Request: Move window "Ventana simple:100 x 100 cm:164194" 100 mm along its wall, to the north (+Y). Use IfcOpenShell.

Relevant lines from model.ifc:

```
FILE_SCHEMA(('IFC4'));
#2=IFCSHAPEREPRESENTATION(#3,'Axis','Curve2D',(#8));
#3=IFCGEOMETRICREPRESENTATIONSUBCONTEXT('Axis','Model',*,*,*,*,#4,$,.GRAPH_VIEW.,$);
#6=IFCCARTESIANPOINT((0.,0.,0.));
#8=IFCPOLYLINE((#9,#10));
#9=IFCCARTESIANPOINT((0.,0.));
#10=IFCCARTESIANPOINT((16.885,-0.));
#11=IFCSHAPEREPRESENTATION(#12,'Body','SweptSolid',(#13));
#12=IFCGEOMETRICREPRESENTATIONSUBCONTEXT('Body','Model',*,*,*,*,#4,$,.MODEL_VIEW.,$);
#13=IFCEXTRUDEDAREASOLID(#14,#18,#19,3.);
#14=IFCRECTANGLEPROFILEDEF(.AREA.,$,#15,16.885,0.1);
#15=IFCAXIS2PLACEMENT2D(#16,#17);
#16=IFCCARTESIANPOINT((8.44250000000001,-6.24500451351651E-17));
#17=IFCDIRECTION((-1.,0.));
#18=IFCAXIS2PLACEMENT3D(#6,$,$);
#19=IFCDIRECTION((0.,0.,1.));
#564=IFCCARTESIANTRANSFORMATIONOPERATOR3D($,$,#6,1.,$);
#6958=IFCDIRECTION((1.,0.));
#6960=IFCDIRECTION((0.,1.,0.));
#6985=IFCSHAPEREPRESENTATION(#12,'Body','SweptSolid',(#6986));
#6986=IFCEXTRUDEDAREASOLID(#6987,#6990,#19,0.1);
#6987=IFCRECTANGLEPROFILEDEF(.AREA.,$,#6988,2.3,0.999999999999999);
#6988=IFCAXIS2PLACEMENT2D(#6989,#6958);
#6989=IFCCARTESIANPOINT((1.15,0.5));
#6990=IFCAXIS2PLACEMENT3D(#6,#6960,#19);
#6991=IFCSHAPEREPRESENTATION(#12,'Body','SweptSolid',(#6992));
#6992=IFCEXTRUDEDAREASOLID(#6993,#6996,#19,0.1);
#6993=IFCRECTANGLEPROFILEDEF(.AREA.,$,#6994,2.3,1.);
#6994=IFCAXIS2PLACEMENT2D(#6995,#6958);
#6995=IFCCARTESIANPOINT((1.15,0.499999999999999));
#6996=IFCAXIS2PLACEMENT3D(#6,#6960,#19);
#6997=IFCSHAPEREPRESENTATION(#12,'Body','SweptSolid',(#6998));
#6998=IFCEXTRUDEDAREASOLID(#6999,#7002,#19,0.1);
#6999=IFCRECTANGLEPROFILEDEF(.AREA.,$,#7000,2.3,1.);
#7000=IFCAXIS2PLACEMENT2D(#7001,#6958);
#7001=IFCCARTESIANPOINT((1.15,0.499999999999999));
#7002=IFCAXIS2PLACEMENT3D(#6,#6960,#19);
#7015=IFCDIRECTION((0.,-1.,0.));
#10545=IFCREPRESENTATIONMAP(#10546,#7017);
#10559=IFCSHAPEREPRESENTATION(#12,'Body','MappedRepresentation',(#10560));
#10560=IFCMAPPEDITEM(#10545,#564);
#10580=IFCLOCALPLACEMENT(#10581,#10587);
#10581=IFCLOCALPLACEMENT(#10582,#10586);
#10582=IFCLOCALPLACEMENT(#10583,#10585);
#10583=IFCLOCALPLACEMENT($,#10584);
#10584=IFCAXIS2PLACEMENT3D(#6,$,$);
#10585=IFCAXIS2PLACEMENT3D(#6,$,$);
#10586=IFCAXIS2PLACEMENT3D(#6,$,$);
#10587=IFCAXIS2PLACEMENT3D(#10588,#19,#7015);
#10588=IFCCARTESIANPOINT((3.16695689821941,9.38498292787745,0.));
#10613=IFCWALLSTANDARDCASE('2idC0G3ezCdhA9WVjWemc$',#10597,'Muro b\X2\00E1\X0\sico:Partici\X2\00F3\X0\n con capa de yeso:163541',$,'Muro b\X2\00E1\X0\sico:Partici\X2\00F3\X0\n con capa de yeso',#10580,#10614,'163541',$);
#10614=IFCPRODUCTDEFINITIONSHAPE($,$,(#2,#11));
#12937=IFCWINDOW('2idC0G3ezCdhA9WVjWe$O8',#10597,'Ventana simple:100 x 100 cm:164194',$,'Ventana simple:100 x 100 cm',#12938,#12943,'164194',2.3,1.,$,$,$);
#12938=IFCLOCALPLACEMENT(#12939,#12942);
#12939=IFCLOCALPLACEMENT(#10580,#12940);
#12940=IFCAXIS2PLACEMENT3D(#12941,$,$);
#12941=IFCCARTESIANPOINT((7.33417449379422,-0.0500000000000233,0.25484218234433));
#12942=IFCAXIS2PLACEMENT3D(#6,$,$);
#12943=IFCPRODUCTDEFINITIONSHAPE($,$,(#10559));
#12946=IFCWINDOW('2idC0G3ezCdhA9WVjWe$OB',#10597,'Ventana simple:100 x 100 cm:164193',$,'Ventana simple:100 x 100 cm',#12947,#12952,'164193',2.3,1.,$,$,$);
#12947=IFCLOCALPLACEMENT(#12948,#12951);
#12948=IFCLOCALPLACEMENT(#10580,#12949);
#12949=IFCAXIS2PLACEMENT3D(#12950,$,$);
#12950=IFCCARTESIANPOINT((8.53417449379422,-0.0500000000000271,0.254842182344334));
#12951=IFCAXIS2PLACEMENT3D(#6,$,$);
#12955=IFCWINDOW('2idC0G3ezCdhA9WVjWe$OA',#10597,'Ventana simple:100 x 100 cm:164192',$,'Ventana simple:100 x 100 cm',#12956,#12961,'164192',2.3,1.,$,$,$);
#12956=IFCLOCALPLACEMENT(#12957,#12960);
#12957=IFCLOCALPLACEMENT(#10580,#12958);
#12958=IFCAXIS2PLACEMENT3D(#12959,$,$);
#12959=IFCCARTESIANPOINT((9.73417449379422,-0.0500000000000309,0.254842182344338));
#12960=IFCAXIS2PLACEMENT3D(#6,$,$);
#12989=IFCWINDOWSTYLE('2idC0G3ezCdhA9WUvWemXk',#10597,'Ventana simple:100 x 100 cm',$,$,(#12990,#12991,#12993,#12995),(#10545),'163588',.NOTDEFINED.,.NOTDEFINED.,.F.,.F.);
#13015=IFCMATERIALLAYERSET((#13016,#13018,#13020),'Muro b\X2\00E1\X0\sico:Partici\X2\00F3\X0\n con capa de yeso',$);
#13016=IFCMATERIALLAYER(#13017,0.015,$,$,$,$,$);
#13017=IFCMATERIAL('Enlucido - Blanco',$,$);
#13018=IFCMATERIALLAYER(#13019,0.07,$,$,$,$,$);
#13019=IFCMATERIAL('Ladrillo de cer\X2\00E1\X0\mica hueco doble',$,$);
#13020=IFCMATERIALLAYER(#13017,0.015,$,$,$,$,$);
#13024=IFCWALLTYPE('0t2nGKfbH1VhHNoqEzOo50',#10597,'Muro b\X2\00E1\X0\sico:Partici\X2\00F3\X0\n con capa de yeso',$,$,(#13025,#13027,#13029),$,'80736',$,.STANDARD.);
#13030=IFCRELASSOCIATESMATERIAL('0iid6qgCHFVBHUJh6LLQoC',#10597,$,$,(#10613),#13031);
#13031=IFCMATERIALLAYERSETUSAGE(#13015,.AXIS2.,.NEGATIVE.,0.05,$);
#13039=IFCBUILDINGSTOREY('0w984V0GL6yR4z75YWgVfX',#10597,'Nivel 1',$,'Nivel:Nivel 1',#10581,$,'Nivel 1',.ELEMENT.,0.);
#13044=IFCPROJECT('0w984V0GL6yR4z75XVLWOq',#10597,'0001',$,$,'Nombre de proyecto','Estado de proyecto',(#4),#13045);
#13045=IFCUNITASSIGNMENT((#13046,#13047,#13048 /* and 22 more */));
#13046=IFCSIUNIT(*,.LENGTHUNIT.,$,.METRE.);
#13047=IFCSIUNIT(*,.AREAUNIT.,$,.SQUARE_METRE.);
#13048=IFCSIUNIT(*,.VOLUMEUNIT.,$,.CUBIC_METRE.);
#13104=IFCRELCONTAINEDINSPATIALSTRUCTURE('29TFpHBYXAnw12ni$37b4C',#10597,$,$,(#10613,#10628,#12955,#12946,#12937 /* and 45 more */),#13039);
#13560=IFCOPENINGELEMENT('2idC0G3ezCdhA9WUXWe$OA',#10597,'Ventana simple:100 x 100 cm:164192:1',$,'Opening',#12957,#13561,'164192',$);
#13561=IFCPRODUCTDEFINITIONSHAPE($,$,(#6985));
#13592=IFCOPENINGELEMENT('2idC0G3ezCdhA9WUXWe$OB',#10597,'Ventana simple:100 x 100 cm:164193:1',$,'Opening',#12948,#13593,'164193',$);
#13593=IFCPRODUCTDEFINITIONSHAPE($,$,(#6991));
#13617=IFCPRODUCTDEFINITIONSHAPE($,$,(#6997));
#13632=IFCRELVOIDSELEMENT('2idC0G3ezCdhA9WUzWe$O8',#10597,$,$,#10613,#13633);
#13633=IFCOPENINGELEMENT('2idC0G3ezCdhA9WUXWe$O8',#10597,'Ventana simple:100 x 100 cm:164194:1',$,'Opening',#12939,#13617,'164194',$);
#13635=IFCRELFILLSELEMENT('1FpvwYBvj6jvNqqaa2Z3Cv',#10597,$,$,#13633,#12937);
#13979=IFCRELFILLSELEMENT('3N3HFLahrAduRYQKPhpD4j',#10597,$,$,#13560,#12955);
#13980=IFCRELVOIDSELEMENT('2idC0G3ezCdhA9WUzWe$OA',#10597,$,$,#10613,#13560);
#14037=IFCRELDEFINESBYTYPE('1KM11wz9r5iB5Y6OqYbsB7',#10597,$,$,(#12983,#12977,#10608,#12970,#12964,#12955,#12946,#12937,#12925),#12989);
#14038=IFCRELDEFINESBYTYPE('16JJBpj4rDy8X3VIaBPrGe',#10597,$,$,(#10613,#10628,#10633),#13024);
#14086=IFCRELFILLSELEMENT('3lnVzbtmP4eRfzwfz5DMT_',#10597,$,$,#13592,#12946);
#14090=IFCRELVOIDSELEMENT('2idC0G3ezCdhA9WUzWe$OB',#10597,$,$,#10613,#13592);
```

```python
import ifcopenshell
import ifcopenshell.api.geometry
import ifcopenshell.util.placement

model = ifcopenshell.open("model.ifc")

window = model.by_guid("2idC0G3ezCdhA9WVjWe$O8")
opening = window.FillsVoids[0].RelatingOpeningElement
wall = opening.VoidsElements[0].RelatingBuildingElement

wall_matrix = ifcopenshell.util.placement.get_local_placement(wall.ObjectPlacement)
shift = wall_matrix[:3, 0] * -0.1
before = ifcopenshell.util.placement.get_local_placement(window.ObjectPlacement)[:3, 3].copy()

# The window is placed relative to its opening, so it follows when the opening moves.
matrix = ifcopenshell.util.placement.get_local_placement(opening.ObjectPlacement)
matrix[:3, 3] += shift
ifcopenshell.api.geometry.edit_object_placement(
    model, product=opening, matrix=matrix, is_si=False, should_transform_children=True
)

after = ifcopenshell.util.placement.get_local_placement(window.ObjectPlacement)[:3, 3]
print("window moved by", (after - before).round(3) + 0.0)

model.write("model-out.ifc")
```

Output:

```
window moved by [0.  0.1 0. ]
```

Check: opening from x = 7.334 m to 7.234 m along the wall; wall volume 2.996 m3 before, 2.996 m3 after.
